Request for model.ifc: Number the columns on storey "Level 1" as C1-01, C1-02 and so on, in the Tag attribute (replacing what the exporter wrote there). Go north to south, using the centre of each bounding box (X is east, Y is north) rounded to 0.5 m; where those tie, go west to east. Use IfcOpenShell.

First a look at what the model holds.

```python
import ifcopenshell
import ifcopenshell.util.element
import ifcopenshell.util.placement

model = ifcopenshell.open("model.ifc")
print(model.schema)
storey = next(s for s in model.by_type("IfcBuildingStorey") if s.Name == "Level 1")
columns = [e for e in ifcopenshell.util.element.get_decomposition(storey) if e.is_a("IfcColumn")]
for e in sorted(columns, key=lambda e: e.id()):
    origin = ifcopenshell.util.placement.get_local_placement(e.ObjectPlacement)[:3, 3]
    print(e.id(), e.Tag, e.Name, origin.round(2) + 0.0, sep=" | ")
```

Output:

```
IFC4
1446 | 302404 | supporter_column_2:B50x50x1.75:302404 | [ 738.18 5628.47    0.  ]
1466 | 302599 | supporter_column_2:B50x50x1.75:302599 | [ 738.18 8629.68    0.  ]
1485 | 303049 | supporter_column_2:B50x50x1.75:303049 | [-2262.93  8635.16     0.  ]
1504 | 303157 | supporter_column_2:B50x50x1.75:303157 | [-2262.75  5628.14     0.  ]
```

```python
import ifcopenshell
import ifcopenshell.geom
import ifcopenshell.util.element
import ifcopenshell.util.shape

model = ifcopenshell.open("model.ifc")
settings = ifcopenshell.geom.settings()
settings.set("use-world-coords", True)


def centre(element):
    shape = ifcopenshell.geom.create_shape(settings, element)
    return ifcopenshell.util.shape.get_bbox_centroid(shape.geometry)


storey = next(s for s in model.by_type("IfcBuildingStorey") if s.Name == "Level 1")
columns = [e for e in ifcopenshell.util.element.get_decomposition(storey) if e.is_a("IfcColumn")]

# Insertion points can sit at a corner or the storey origin, so sort by the geometry (in metres).
centres = {e: centre(e) for e in columns}
columns.sort(key=lambda e: (-round(centres[e][1] / 0.5), centres[e][0]))

for i, e in enumerate(columns, start=1):
    number = f"C1-{i:02d}"
    e.Tag = number
    print(e.id(), number)

model.write("model_rev.ifc")
```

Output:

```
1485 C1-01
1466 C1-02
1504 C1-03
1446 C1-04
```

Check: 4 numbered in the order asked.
